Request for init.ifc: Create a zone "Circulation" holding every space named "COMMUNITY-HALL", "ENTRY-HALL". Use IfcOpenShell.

First a look at what the model holds.

```python
import ifcopenshell

model = ifcopenshell.open("init.ifc")
print(model.schema)
seen = {}
for space in model.by_type("IfcSpace"):
    seen[space.Name] = seen.get(space.Name, 0) + 1
for name, count in sorted(seen.items(), key=str):
    print(count, "x", name)
print("zones:", [z.Name for z in model.by_type("IfcZone")][:20])
```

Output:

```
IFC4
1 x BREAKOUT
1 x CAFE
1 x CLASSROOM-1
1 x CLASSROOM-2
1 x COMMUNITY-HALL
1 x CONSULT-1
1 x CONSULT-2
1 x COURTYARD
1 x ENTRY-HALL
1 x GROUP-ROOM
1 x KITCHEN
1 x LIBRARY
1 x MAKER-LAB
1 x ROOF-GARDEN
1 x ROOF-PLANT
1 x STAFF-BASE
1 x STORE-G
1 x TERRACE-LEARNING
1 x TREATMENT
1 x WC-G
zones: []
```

```python
import ifcopenshell
import ifcopenshell.api.group
import ifcopenshell.api.root

model = ifcopenshell.open("init.ifc")

names = {"COMMUNITY-HALL", "ENTRY-HALL"}
spaces = [s for s in model.by_type("IfcSpace") if s.Name in names]

zone = ifcopenshell.api.root.create_entity(model, ifc_class="IfcZone", name="Circulation")
ifcopenshell.api.group.assign_group(model, products=spaces, group=zone)
print(len(spaces), "spaces in", zone.Name)

model.write("init_v2.ifc")
```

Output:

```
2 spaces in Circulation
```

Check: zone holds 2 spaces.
